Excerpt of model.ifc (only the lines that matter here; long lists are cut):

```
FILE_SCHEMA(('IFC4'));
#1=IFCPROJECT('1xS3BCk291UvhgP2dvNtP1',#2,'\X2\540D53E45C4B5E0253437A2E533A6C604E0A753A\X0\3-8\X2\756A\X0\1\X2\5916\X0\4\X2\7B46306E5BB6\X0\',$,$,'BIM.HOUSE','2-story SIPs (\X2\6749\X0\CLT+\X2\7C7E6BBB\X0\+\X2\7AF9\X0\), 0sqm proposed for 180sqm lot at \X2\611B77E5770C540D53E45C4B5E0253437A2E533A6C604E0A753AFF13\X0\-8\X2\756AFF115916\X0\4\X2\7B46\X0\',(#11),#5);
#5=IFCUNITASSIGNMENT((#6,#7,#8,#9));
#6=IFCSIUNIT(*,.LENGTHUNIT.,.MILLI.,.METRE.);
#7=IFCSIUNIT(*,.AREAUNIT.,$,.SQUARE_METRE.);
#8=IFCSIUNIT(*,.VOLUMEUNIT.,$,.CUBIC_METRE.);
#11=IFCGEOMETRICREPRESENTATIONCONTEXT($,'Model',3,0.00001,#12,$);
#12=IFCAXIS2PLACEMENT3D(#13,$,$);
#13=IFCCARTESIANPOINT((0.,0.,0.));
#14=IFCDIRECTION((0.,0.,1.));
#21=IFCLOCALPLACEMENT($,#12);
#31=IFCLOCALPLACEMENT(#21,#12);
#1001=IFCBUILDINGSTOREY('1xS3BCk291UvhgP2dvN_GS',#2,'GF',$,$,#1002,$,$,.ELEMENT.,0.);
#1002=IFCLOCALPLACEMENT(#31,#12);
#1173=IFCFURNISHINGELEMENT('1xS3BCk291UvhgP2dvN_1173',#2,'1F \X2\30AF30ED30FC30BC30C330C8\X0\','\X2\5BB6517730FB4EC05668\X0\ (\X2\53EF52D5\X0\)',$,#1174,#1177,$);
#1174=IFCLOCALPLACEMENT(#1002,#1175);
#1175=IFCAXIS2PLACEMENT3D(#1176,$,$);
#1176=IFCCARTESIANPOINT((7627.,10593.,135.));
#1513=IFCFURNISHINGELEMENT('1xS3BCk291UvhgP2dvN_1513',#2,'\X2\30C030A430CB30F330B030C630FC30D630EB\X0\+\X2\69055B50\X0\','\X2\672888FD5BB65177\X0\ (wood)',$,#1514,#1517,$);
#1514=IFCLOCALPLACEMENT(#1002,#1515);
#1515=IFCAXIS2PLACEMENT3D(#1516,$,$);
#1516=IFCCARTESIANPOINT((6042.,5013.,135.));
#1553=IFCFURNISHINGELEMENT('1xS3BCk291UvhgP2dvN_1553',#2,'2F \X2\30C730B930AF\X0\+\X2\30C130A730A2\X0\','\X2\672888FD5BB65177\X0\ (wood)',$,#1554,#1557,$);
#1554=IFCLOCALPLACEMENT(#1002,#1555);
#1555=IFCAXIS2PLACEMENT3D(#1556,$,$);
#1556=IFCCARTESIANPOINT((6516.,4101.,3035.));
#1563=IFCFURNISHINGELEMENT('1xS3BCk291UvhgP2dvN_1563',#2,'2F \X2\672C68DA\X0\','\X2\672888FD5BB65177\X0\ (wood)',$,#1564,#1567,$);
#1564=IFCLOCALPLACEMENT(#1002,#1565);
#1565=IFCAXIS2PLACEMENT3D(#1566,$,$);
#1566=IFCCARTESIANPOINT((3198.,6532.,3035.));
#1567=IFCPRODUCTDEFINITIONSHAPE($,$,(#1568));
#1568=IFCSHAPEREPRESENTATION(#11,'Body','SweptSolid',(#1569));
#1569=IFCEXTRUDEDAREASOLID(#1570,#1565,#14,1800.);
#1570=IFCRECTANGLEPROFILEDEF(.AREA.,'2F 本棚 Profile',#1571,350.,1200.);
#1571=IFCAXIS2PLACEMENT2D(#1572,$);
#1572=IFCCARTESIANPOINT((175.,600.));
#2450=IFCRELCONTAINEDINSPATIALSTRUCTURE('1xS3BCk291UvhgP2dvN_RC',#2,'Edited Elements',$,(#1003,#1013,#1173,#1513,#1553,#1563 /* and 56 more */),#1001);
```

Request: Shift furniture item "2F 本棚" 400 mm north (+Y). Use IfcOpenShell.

```python
import ifcopenshell
import ifcopenshell.api.geometry
import ifcopenshell.util.placement

model = ifcopenshell.open("model.ifc")

item = model.by_id(1563)
matrix = ifcopenshell.util.placement.get_local_placement(item.ObjectPlacement)
matrix[1, 3] += 400.0
ifcopenshell.api.geometry.edit_object_placement(model, product=item, matrix=matrix, is_si=False)

print(ifcopenshell.util.placement.get_local_placement(item.ObjectPlacement).round(3) + 0.0)

model.write("model_rev.ifc")
```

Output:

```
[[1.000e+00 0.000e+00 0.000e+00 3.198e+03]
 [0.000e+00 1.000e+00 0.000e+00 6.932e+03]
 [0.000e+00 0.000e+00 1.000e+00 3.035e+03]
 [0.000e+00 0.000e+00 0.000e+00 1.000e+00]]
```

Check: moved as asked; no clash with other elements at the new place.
